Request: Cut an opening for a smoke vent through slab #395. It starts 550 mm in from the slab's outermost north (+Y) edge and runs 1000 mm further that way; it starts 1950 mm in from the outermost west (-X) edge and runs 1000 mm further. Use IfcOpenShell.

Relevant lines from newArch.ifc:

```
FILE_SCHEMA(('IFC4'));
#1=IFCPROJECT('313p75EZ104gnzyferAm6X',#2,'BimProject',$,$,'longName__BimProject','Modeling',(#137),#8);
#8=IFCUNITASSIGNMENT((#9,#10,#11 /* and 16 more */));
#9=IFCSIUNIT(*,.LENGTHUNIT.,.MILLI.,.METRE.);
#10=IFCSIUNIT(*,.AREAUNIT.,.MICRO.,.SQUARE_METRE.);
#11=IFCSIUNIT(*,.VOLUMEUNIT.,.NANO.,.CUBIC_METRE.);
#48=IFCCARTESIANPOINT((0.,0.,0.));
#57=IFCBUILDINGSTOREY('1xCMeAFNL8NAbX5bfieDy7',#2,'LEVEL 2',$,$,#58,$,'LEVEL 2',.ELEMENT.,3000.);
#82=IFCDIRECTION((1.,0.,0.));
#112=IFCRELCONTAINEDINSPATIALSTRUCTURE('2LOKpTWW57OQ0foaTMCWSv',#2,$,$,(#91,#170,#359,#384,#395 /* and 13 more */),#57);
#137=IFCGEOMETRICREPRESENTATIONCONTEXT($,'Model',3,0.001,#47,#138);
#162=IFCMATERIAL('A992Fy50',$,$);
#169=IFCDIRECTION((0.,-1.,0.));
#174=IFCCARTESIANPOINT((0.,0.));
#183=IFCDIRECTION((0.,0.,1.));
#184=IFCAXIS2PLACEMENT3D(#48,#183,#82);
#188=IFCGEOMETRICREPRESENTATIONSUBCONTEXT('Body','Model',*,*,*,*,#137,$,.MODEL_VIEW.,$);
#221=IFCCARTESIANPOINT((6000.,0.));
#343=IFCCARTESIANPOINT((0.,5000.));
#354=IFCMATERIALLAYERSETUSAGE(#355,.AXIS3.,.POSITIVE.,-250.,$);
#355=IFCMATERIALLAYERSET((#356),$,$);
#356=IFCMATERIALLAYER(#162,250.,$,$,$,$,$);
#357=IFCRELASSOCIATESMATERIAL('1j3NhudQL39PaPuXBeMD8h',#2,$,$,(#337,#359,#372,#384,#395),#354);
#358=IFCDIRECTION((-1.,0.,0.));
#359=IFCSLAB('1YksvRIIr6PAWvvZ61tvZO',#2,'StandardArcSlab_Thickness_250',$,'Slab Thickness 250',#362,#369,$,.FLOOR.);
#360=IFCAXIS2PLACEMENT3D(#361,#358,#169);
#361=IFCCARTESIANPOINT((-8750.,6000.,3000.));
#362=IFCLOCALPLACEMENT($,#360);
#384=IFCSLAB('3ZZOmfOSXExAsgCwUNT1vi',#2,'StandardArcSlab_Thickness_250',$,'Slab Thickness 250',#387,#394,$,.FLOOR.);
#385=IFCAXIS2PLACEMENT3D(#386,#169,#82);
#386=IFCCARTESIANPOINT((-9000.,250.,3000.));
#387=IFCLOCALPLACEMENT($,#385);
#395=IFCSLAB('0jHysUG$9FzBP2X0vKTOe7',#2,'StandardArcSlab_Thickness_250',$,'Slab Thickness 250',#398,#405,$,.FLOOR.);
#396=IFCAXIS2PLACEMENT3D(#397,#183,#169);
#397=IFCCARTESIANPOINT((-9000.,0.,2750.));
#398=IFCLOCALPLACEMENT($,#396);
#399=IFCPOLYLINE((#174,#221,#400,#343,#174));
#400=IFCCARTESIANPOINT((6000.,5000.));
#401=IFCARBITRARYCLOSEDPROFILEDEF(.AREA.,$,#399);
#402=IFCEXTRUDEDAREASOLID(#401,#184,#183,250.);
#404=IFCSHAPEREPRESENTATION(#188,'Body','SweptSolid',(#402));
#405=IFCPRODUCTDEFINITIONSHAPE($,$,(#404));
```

```python
import numpy as np
import ifcopenshell
import ifcopenshell.api.feature
import ifcopenshell.api.geometry
import ifcopenshell.api.root
import ifcopenshell.geom
import ifcopenshell.util.placement
import ifcopenshell.util.representation
import ifcopenshell.util.shape
import ifcopenshell.util.unit

model = ifcopenshell.open("newArch.ifc")
unit_scale = ifcopenshell.util.unit.calculate_unit_scale(model)
settings = ifcopenshell.geom.settings()


def volume(element):
    """Net volume in cubic metres, openings subtracted."""
    shape = ifcopenshell.geom.create_shape(settings, element)
    return ifcopenshell.util.shape.get_volume(shape.geometry)


slab = model.by_id(395)
before = volume(slab)

# Extent in the slab's own axes, in metres. The edges named are its -X and -Y sides.
slab_shape = ifcopenshell.geom.create_shape(settings, slab)
vertices = ifcopenshell.util.shape.get_vertices(slab_shape.geometry)
x_min, y_min, bottom = vertices.min(axis=0)
top = vertices[:, 2].max()

opening = ifcopenshell.api.root.create_entity(model, ifc_class="IfcOpeningElement", name="Smoke vent opening", predefined_type="OPENING")
context = ifcopenshell.util.representation.get_context(model, "Model", "Body", "MODEL_VIEW")
width, depth = 1, 1
outline = [(0.0, 0.0), (width, 0.0), (width, depth), (0.0, depth), (0.0, 0.0)]
# Overshoot both faces by 50 mm so the cut is clean.
shape = ifcopenshell.api.geometry.add_slab_representation(
    model, context=context, depth=top - bottom + 0.1, polyline=outline
)
ifcopenshell.api.geometry.assign_representation(model, product=opening, representation=shape)

matrix = ifcopenshell.util.placement.get_local_placement(slab.ObjectPlacement)
matrix[:, 3] = matrix @ np.append(np.array([x_min + 0.55, y_min + 1.95, bottom - 0.05]) / unit_scale, 1.0)
ifcopenshell.api.geometry.edit_object_placement(model, product=opening, matrix=matrix, is_si=False)
ifcopenshell.api.feature.add_feature(model, feature=opening, element=slab)

after = volume(slab)

print(f"slab volume {before:.3f} -> {after:.3f} m3")

model.write("newArch_updated.ifc")
```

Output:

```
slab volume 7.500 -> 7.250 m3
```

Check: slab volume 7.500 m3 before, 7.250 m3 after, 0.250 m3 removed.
